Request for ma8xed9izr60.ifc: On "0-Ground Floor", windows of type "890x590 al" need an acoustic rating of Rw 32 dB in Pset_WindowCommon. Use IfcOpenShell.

First a look at what the model holds.

```python
import ifcopenshell
import ifcopenshell.util.element

model = ifcopenshell.open("ma8xed9izr60.ifc")
print(model.schema)
storey = next(s for s in model.by_type("IfcBuildingStorey") if s.Name == "0-Ground Floor")
windows = [e for e in ifcopenshell.util.element.get_decomposition(storey) if e.is_a("IfcWindow")]
seen = {}
for e in windows:
    element_type = ifcopenshell.util.element.get_type(e)
    key = (element_type.Name if element_type != e and element_type else None, ifcopenshell.util.element.get_pset(e, "Pset_WindowCommon", "AcousticRating"))
    seen[key] = seen.get(key, 0) + 1
for (name, value), count in sorted(seen.items(), key=str):
    print(count, "x", name, "|", value)
```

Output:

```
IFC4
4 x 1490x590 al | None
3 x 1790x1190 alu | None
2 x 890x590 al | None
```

```python
import ifcopenshell
import ifcopenshell.api.pset
import ifcopenshell.util.element

model = ifcopenshell.open("ma8xed9izr60.ifc")

storey = next(s for s in model.by_type("IfcBuildingStorey") if s.Name == "0-Ground Floor")
windows = [e for e in ifcopenshell.util.element.get_decomposition(storey) if e.is_a("IfcWindow")]

count = 0
for e in windows:
    element_type = ifcopenshell.util.element.get_type(e)
    if element_type in (None, e) or element_type.Name != "890x590 al":
        continue
    # add_pset returns the element's existing set when there is one.
    pset = ifcopenshell.api.pset.add_pset(model, product=e, name="Pset_WindowCommon")
    ifcopenshell.api.pset.edit_pset(model, pset=pset, properties={"AcousticRating": "Rw 32 dB"})
    count += 1

print(count, "windows updated")

model.write("ma8xed9izr60_rev.ifc")
```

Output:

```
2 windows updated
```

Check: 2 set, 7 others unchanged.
